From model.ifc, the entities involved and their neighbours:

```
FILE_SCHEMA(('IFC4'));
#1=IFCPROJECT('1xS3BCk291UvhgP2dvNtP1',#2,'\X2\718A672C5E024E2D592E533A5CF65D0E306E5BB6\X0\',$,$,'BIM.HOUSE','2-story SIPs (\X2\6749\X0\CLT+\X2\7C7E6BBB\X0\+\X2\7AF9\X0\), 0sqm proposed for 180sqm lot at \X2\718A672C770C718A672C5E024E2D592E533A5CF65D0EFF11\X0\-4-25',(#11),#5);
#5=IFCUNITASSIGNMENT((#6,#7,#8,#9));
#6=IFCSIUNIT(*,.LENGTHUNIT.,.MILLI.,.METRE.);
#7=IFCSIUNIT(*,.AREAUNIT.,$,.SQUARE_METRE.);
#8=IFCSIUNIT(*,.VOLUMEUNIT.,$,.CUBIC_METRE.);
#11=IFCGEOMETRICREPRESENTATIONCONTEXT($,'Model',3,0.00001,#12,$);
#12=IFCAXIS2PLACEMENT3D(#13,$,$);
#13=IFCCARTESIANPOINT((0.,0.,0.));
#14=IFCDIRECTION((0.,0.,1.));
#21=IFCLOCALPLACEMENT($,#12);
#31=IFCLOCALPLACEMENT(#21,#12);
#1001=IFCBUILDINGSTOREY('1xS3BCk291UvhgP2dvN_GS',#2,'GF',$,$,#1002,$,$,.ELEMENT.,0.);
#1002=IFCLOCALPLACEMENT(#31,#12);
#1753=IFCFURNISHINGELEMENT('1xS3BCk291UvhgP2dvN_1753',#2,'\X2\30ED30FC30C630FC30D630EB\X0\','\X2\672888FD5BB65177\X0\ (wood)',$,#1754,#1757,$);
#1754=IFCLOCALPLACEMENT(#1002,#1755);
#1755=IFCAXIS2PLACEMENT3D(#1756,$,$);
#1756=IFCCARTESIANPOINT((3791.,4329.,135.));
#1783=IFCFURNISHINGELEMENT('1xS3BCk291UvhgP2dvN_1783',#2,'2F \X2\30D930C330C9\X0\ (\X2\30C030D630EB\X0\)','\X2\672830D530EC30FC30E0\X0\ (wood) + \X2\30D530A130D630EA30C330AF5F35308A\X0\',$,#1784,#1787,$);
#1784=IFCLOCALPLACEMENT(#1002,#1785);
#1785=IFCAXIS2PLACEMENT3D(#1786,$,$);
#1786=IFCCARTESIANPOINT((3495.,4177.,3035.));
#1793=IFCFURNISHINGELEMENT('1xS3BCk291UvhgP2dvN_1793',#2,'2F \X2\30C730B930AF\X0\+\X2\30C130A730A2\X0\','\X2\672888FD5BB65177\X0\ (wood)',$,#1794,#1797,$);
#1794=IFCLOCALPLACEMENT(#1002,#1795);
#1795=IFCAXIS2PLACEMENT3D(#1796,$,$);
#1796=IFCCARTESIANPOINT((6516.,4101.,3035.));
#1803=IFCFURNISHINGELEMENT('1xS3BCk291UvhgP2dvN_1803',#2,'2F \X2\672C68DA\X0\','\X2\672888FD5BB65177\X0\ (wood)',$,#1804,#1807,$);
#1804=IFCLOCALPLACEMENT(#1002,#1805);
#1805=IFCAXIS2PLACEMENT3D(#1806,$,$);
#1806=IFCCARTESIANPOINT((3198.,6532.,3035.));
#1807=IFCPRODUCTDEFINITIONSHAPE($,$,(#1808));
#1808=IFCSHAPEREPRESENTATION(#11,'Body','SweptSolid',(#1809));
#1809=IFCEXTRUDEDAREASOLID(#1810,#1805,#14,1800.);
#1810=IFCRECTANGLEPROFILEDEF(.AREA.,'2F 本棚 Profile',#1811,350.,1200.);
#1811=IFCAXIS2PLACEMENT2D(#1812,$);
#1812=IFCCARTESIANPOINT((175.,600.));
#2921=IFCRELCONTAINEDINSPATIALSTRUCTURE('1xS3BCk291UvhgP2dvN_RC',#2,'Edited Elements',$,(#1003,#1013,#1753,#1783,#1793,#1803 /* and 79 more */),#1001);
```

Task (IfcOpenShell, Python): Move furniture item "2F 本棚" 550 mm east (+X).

```python
import ifcopenshell
import ifcopenshell.api.geometry
import ifcopenshell.util.placement

model = ifcopenshell.open("model.ifc")

item = model.by_id(1803)
matrix = ifcopenshell.util.placement.get_local_placement(item.ObjectPlacement)
matrix[0, 3] += 550.0
ifcopenshell.api.geometry.edit_object_placement(model, product=item, matrix=matrix, is_si=False)

print(ifcopenshell.util.placement.get_local_placement(item.ObjectPlacement).round(3) + 0.0)

model.write("model_rev.ifc")
```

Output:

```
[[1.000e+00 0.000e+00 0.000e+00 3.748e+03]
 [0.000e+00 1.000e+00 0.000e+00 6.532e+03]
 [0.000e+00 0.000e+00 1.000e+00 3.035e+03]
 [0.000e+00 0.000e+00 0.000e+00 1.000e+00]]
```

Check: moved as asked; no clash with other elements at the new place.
